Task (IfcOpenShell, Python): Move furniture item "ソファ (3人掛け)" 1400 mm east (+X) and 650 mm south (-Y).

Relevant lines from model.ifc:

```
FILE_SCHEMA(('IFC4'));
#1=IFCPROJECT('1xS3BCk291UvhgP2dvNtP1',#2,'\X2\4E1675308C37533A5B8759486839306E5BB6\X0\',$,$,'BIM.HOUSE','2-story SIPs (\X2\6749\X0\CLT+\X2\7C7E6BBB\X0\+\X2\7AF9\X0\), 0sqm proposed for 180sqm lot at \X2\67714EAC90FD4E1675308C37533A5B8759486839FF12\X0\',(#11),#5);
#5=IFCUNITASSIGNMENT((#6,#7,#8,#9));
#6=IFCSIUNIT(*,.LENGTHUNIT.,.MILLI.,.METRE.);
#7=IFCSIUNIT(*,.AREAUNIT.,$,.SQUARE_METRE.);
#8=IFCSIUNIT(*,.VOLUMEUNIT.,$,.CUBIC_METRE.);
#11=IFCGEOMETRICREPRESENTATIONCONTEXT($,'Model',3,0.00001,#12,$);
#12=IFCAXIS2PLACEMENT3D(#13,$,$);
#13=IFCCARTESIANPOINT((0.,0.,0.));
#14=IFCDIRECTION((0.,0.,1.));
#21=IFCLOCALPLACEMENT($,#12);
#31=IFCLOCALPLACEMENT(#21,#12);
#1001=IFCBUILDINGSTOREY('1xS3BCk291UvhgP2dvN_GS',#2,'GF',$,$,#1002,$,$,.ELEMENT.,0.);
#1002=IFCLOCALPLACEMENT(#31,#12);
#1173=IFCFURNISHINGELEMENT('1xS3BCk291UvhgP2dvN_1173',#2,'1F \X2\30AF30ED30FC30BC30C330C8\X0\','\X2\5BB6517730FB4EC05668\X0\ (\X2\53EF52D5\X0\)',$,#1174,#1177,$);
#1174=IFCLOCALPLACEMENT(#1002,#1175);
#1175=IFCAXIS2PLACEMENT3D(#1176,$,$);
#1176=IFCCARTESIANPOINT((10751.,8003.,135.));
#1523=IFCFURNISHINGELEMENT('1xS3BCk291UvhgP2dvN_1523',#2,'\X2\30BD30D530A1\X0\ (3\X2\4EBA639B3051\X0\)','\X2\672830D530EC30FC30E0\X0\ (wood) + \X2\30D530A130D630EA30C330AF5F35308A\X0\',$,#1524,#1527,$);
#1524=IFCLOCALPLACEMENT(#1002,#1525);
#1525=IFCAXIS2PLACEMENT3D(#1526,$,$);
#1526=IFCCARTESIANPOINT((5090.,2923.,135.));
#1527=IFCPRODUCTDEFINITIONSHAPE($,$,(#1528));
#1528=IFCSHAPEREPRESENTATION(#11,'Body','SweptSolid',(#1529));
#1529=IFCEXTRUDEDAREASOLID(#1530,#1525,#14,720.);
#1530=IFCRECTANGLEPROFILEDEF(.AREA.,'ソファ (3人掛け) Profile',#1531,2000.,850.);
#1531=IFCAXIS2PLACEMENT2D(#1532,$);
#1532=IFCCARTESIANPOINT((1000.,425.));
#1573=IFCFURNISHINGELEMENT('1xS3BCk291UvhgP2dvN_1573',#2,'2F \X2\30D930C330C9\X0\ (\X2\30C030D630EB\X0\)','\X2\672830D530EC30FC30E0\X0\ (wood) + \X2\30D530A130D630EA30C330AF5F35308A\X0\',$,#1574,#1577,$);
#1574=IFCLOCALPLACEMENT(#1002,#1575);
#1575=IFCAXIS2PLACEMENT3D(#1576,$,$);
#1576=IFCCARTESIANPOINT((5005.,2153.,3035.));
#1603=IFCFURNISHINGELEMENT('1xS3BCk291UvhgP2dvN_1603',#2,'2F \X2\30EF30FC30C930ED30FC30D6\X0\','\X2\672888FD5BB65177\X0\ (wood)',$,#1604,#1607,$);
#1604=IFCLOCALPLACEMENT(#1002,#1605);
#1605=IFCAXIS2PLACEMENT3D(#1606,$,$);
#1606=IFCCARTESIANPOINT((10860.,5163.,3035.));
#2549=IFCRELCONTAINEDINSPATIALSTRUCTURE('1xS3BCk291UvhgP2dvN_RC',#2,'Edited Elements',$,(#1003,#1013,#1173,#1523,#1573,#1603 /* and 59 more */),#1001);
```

```python
import ifcopenshell
import ifcopenshell.api.geometry
import ifcopenshell.util.placement

model = ifcopenshell.open("model.ifc")

item = model.by_guid("1xS3BCk291UvhgP2dvN_1523")
matrix = ifcopenshell.util.placement.get_local_placement(item.ObjectPlacement)
matrix[0, 3] += 1400.0
matrix[1, 3] -= 650.0
ifcopenshell.api.geometry.edit_object_placement(model, product=item, matrix=matrix, is_si=False)

print(ifcopenshell.util.placement.get_local_placement(item.ObjectPlacement).round(3) + 0.0)

model.write("model_v2.ifc")
```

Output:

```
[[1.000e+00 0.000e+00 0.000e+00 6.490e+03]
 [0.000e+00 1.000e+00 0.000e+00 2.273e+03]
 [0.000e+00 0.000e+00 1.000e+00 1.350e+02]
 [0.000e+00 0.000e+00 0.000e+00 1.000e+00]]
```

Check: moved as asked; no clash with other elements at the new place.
